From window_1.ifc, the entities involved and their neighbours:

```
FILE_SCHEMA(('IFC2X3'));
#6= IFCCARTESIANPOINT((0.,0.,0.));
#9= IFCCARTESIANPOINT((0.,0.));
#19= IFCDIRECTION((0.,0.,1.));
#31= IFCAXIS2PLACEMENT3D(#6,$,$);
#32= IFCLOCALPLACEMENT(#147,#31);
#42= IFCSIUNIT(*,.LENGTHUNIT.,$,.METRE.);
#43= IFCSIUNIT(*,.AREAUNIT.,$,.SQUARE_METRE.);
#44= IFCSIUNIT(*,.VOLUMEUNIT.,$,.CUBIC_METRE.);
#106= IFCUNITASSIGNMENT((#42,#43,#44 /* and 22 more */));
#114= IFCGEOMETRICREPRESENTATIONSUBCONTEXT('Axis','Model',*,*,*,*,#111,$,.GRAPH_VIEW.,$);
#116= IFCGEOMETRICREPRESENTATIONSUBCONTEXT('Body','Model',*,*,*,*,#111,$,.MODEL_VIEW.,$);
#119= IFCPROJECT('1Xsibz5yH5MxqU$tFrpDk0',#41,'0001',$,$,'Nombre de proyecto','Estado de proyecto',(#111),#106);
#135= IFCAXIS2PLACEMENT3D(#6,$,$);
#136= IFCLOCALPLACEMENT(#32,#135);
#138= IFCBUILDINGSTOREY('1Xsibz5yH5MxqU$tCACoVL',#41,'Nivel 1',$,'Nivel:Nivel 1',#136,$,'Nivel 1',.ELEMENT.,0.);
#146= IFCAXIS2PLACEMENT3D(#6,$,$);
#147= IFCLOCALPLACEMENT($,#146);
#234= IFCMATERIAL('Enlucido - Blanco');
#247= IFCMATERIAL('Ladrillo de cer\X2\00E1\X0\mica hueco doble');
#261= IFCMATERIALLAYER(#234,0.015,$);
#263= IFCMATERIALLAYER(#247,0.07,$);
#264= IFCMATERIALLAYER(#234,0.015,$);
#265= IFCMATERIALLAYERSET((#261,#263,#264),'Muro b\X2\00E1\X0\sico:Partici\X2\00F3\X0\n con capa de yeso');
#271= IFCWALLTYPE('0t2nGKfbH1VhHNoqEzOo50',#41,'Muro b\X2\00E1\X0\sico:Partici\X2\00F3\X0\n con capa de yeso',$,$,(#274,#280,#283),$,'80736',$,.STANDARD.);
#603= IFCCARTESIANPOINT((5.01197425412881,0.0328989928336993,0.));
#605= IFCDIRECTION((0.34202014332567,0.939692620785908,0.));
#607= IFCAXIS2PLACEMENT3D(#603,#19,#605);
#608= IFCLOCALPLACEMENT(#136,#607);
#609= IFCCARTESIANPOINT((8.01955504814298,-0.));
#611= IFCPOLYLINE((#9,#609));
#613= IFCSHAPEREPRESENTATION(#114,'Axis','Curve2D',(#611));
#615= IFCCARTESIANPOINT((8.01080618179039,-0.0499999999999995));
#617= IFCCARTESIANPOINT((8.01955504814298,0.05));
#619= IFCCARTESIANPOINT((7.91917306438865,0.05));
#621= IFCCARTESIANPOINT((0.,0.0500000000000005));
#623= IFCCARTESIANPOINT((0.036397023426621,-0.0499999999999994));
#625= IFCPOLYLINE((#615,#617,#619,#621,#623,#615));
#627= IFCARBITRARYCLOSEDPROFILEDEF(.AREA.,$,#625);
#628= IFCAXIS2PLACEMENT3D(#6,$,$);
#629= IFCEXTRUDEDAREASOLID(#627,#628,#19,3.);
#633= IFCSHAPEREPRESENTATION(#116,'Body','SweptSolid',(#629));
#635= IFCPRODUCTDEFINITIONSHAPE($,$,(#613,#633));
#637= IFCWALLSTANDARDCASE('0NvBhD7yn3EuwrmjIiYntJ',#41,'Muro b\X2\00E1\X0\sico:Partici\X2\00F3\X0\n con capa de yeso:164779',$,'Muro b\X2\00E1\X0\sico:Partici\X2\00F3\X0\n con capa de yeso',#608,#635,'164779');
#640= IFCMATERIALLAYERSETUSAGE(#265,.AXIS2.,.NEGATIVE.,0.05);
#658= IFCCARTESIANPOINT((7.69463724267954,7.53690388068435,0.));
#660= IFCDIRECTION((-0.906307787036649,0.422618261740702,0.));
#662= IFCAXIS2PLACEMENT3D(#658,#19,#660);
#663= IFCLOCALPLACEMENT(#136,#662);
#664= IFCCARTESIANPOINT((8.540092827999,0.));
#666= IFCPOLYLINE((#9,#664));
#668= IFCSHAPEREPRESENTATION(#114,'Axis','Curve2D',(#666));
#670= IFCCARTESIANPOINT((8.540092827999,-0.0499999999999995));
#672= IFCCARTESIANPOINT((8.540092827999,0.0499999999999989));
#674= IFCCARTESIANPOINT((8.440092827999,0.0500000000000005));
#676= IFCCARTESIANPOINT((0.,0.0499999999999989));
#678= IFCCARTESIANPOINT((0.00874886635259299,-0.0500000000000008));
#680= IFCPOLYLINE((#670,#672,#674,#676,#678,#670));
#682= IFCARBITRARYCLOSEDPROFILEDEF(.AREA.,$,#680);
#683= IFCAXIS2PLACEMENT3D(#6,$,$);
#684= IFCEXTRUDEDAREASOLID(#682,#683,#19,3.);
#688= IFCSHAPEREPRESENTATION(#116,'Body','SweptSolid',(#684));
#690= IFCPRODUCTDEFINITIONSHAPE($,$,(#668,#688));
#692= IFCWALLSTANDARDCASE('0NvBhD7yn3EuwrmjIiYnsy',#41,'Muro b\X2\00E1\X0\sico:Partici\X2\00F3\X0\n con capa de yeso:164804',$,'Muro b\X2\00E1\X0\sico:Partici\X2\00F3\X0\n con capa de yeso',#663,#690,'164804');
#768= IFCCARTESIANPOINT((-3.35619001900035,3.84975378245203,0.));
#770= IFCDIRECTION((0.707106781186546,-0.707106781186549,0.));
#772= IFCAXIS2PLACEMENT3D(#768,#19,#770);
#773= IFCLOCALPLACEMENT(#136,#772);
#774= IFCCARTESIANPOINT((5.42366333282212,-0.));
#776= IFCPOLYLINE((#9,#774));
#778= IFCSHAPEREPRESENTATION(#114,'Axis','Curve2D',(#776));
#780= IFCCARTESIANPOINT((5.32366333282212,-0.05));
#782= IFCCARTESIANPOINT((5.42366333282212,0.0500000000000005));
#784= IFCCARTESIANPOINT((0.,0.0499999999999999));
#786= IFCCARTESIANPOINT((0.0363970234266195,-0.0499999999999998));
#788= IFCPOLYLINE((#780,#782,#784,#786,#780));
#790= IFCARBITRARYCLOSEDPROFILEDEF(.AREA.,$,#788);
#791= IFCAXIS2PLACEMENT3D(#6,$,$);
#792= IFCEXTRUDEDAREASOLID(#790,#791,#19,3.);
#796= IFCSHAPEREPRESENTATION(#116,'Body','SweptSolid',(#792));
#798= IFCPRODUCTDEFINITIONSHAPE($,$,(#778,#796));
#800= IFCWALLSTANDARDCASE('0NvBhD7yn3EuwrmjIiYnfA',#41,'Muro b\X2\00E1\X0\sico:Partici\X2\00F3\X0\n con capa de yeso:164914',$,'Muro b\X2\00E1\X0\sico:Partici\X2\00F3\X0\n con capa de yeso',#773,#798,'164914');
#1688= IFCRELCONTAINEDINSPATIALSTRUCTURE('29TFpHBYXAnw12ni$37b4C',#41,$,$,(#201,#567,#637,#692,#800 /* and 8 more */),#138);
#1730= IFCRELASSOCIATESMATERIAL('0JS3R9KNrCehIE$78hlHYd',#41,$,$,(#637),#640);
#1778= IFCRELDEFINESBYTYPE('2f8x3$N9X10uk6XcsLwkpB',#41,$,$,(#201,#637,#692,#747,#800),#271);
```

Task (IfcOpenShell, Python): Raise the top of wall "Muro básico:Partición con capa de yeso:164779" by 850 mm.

```python
import ifcopenshell
import ifcopenshell.geom
import ifcopenshell.util.representation
import ifcopenshell.util.shape
import ifcopenshell.util.unit

model = ifcopenshell.open("window_1.ifc")
unit_scale = ifcopenshell.util.unit.calculate_unit_scale(model)
settings = ifcopenshell.geom.settings()


def volume(element):
    """Net volume in cubic metres, openings subtracted."""
    shape = ifcopenshell.geom.create_shape(settings, element)
    return ifcopenshell.util.shape.get_volume(shape.geometry)


wall = model.by_guid("0NvBhD7yn3EuwrmjIiYntJ")
before = volume(wall)

body = ifcopenshell.util.representation.get_representation(wall, "Model", "Body")
solid = body.Items[0]
old_height = solid.Depth
solid.Depth += 0.85 / unit_scale
after = volume(wall)

print(f"height {old_height:g} -> {solid.Depth:g}, volume {before:.3f} -> {after:.3f} m3")

model.write("window_1-out.ifc")
```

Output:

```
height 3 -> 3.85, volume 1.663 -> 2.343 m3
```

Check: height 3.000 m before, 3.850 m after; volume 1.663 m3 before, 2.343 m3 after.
